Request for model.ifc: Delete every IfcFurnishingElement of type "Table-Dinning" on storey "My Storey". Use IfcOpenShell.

First a look at what the model holds.

```python
import ifcopenshell
import ifcopenshell.util.element

model = ifcopenshell.open("model.ifc")
print(model.schema)
storey = next(s for s in model.by_type("IfcBuildingStorey") if s.Name == "My Storey")
furniture = [e for e in ifcopenshell.util.element.get_decomposition(storey) if e.is_a("IfcFurnishingElement")]
seen = {}
for e in furniture:
    element_type = ifcopenshell.util.element.get_type(e)
    name = element_type.Name if element_type not in (None, e) else None
    seen[name] = seen.get(name, 0) + 1
for name, count in sorted(seen.items(), key=str):
    print(count, "x", name)
```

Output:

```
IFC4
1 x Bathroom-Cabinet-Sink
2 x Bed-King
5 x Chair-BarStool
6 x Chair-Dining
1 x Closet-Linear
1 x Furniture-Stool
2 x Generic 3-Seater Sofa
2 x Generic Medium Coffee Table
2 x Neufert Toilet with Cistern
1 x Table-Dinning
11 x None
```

```python
import ifcopenshell
import ifcopenshell.api.root
import ifcopenshell.util.element

model = ifcopenshell.open("model.ifc")

storey = next(s for s in model.by_type("IfcBuildingStorey") if s.Name == "My Storey")
furniture = [e for e in ifcopenshell.util.element.get_decomposition(storey) if e.is_a("IfcFurnishingElement")]
targets = [e for e in furniture if (t := ifcopenshell.util.element.get_type(e)) not in (None, e) and t.Name == "Table-Dinning"]

for e in targets:
    ifcopenshell.api.root.remove_product(model, product=e)
print(len(targets), "removed")

model.write("model-out.ifc")
```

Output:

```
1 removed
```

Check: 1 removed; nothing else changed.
